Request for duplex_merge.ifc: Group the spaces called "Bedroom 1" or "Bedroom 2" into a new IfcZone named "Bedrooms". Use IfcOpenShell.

First a look at what the model holds.

```python
import ifcopenshell

model = ifcopenshell.open("duplex_merge.ifc")
print(model.schema)
seen = {}
for space in model.by_type("IfcSpace"):
    seen[space.LongName] = seen.get(space.LongName, 0) + 1
for name, count in sorted(seen.items(), key=str):
    print(count, "x", name)
print("zones:", [z.Name for z in model.by_type("IfcZone")][:20])
```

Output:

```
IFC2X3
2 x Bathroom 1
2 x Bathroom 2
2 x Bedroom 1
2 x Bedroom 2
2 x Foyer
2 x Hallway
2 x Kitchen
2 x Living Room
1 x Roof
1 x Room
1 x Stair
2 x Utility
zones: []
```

```python
import ifcopenshell
import ifcopenshell.api.group
import ifcopenshell.api.root

model = ifcopenshell.open("duplex_merge.ifc")

names = {"Bedroom 1", "Bedroom 2"}
spaces = [s for s in model.by_type("IfcSpace") if s.LongName in names]

zone = ifcopenshell.api.root.create_entity(model, ifc_class="IfcZone", name="Bedrooms")
ifcopenshell.api.group.assign_group(model, products=spaces, group=zone)
print(len(spaces), "spaces in", zone.Name)

model.write("duplex_merge_v2.ifc")
```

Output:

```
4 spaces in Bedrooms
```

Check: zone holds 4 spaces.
